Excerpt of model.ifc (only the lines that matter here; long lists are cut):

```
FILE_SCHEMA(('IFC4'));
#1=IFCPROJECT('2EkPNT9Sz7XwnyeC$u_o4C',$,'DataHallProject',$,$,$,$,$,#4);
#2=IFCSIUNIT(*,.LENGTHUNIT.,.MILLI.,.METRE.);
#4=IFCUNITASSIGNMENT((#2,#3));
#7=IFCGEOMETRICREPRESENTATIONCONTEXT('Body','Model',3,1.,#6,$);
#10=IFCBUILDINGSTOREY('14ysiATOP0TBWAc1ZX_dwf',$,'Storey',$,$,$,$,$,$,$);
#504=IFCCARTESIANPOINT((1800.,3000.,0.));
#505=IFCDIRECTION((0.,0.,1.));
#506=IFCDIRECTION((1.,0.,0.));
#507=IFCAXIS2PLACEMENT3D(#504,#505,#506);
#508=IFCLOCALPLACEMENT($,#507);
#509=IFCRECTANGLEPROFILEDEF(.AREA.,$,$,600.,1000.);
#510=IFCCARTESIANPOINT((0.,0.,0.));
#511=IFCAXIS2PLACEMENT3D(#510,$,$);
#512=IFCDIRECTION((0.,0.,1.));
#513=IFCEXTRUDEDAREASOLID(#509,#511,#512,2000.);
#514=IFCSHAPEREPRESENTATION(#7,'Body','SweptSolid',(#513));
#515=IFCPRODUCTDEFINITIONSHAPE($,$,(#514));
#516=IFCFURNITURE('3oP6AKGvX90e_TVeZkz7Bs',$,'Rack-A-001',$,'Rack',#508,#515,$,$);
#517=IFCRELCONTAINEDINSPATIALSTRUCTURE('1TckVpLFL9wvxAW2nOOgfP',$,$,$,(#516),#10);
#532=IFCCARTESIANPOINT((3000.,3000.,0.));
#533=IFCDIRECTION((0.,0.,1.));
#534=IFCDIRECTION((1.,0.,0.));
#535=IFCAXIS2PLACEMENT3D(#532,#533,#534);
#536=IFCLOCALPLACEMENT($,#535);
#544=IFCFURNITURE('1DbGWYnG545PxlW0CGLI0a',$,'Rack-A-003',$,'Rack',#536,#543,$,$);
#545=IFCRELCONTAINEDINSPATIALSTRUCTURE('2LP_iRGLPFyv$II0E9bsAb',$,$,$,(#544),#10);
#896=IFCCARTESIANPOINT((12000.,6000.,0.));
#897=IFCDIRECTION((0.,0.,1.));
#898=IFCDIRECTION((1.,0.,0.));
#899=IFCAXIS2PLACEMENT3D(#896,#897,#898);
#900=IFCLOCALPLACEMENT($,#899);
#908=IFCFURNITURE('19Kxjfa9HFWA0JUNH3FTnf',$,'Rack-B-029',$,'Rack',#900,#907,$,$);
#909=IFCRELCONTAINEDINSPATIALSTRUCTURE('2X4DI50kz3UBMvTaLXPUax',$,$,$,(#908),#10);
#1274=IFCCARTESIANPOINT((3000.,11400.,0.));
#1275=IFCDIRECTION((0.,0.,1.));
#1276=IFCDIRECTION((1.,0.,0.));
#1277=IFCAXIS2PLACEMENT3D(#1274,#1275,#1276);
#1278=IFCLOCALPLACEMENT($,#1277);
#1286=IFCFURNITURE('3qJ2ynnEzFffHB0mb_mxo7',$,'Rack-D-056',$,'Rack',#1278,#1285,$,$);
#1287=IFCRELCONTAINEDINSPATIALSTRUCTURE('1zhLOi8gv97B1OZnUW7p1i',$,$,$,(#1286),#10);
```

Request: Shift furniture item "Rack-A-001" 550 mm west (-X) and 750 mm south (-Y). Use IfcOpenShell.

```python
import ifcopenshell
import ifcopenshell.api.geometry
import ifcopenshell.util.placement
import ifcopenshell.util.unit

model = ifcopenshell.open("model.ifc")
unit_scale = ifcopenshell.util.unit.calculate_unit_scale(model)

item = model.by_guid("3oP6AKGvX90e_TVeZkz7Bs")
matrix = ifcopenshell.util.placement.get_local_placement(item.ObjectPlacement)
matrix[0, 3] -= 0.55 / unit_scale
matrix[1, 3] -= 0.75 / unit_scale
ifcopenshell.api.geometry.edit_object_placement(model, product=item, matrix=matrix, is_si=False)

print(ifcopenshell.util.placement.get_local_placement(item.ObjectPlacement).round(3) + 0.0)

model.write("model_updated.ifc")
```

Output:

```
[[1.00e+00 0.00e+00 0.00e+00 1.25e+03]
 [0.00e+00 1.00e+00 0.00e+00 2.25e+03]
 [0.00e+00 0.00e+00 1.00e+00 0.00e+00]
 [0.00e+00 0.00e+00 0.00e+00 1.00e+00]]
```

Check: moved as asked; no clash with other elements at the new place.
